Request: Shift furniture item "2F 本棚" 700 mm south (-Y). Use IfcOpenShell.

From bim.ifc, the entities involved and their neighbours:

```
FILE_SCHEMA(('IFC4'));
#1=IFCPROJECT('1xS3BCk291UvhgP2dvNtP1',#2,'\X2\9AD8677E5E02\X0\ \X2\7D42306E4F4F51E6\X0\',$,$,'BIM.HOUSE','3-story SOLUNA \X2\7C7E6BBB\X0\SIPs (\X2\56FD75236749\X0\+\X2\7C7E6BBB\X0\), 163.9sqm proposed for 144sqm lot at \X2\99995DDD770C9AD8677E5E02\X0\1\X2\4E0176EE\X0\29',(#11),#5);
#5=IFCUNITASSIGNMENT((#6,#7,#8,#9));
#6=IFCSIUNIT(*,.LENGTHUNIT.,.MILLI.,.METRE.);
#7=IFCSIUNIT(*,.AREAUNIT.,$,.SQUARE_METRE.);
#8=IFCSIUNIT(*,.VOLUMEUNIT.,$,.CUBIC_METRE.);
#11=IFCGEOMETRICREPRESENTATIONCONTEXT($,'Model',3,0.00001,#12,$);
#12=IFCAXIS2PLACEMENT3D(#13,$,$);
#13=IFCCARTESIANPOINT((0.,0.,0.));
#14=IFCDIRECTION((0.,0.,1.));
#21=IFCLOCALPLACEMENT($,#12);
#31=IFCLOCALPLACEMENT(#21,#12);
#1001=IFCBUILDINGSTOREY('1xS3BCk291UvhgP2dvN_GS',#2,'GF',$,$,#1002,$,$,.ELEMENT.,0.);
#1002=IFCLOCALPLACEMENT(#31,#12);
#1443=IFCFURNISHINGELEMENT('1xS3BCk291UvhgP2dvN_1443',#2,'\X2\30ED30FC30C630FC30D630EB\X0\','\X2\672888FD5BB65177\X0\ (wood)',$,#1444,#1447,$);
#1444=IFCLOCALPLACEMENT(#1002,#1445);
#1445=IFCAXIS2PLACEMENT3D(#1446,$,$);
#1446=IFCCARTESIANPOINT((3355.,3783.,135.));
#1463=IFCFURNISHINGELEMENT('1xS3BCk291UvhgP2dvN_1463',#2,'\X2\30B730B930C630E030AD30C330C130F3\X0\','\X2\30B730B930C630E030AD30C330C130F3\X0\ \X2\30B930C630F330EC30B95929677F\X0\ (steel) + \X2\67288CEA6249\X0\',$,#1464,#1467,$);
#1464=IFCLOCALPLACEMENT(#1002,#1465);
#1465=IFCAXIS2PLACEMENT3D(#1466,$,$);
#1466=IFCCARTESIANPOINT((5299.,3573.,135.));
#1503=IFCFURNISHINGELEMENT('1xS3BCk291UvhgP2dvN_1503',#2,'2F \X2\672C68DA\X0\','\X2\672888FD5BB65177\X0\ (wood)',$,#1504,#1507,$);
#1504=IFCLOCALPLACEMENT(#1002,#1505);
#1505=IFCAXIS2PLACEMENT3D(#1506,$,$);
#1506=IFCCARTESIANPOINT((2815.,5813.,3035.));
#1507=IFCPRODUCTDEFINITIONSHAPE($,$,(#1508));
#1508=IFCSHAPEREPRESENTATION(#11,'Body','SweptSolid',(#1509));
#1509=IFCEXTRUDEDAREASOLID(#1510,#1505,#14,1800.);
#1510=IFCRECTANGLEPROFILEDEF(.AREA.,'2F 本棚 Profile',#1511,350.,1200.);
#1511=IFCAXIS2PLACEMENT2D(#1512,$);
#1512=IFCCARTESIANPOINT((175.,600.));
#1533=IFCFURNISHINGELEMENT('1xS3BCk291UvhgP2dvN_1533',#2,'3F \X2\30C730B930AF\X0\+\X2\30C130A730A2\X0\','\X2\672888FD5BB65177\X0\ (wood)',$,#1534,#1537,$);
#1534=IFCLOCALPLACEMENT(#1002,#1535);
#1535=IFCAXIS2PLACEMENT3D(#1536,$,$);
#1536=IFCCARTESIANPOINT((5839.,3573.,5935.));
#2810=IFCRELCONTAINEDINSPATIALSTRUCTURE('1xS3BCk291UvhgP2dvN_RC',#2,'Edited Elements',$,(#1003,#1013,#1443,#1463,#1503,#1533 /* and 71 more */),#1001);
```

```python
import ifcopenshell
import ifcopenshell.api.geometry
import ifcopenshell.util.placement

model = ifcopenshell.open("bim.ifc")

item = model.by_guid("1xS3BCk291UvhgP2dvN_1503")
matrix = ifcopenshell.util.placement.get_local_placement(item.ObjectPlacement)
matrix[1, 3] -= 700.0
ifcopenshell.api.geometry.edit_object_placement(model, product=item, matrix=matrix, is_si=False)

print(ifcopenshell.util.placement.get_local_placement(item.ObjectPlacement).round(3) + 0.0)

model.write("bim_updated.ifc")
```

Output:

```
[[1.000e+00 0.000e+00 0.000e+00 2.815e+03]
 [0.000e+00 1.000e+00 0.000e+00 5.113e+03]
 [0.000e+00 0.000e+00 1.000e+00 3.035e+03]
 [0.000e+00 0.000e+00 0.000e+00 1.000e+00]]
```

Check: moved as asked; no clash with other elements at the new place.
